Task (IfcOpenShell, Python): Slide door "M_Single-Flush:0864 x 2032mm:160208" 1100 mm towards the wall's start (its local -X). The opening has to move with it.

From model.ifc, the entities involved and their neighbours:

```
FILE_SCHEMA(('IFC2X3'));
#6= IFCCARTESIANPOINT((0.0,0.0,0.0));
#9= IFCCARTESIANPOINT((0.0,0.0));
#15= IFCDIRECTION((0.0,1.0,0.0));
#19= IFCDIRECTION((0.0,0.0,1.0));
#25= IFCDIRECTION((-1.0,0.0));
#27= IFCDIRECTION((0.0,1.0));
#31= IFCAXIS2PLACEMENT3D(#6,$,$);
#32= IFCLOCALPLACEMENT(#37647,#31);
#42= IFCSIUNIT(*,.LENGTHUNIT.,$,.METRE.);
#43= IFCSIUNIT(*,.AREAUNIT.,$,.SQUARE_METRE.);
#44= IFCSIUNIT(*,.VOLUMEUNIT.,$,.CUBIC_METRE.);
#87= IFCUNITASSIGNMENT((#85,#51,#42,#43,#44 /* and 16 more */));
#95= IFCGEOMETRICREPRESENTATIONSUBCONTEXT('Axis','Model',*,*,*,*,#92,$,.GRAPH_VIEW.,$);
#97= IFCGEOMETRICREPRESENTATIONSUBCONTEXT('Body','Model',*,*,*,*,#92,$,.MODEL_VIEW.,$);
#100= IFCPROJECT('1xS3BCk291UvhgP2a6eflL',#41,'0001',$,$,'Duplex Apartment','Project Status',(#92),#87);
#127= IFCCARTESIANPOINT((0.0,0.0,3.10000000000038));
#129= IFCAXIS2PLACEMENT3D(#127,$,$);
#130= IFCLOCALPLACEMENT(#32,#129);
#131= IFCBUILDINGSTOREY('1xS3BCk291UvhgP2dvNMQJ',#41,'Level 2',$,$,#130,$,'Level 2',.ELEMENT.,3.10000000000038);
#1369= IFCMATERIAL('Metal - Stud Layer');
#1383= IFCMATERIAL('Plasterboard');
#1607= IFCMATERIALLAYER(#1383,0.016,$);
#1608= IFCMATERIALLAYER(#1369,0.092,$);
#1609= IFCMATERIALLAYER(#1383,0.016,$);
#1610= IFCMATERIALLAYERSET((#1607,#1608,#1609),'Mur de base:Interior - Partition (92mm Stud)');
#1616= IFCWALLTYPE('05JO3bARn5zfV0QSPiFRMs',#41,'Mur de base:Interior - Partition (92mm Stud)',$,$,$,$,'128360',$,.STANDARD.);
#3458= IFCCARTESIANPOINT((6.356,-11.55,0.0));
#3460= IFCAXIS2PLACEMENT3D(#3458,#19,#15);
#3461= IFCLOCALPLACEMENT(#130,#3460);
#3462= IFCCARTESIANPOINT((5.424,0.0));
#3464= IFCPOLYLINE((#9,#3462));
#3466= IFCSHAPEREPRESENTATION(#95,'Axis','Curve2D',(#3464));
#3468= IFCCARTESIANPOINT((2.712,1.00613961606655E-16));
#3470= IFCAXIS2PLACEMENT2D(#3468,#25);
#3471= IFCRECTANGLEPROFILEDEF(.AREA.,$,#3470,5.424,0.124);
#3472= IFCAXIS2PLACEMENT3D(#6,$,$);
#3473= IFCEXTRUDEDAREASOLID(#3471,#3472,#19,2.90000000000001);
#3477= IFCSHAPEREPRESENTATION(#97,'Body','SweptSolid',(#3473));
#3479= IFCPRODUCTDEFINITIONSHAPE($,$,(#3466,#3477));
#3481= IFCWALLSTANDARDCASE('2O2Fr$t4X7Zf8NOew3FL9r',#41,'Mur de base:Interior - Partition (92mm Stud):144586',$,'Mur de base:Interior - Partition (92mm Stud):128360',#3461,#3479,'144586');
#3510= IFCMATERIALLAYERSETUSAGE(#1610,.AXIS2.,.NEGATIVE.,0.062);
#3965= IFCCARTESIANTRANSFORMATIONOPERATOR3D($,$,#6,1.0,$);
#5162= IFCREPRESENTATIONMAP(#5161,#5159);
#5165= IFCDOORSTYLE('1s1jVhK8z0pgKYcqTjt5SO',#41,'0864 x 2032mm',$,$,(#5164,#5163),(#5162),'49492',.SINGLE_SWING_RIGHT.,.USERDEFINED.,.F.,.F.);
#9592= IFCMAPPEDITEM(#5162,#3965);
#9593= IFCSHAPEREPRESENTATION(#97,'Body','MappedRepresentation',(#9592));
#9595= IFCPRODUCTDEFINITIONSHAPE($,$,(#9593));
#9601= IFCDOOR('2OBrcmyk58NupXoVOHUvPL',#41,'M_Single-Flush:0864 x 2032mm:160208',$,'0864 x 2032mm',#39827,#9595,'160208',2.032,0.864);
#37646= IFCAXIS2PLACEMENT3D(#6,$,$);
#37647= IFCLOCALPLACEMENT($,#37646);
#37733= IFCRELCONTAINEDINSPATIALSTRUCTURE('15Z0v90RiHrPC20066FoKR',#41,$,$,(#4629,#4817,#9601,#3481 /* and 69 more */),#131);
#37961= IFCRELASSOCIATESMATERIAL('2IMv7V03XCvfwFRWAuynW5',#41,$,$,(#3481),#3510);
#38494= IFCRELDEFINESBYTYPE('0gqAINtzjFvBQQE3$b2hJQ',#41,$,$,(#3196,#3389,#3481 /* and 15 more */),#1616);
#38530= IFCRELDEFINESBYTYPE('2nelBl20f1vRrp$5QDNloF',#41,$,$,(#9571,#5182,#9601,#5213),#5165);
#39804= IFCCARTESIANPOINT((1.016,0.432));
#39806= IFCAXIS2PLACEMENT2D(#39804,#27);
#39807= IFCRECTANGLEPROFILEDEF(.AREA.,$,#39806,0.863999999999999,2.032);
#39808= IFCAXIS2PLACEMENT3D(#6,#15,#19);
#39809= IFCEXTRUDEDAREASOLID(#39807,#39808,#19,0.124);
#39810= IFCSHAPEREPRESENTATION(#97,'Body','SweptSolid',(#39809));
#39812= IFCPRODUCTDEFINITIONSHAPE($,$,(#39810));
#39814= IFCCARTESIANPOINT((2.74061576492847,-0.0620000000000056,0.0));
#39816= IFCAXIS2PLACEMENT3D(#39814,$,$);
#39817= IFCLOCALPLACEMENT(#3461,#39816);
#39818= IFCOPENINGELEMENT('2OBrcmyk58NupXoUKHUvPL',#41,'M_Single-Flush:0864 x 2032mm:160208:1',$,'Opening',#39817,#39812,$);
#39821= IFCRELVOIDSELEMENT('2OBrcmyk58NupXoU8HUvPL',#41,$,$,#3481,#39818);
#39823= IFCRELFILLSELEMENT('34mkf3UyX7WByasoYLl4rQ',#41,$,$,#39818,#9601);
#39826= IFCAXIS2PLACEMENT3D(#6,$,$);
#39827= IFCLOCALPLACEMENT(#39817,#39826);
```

```python
import ifcopenshell
import ifcopenshell.api.geometry
import ifcopenshell.util.placement
import ifcopenshell.util.unit

model = ifcopenshell.open("model.ifc")
unit_scale = ifcopenshell.util.unit.calculate_unit_scale(model)

door = model.by_guid("2OBrcmyk58NupXoVOHUvPL")
opening = door.FillsVoids[0].RelatingOpeningElement
wall = opening.VoidsElements[0].RelatingBuildingElement

wall_matrix = ifcopenshell.util.placement.get_local_placement(wall.ObjectPlacement)
shift = wall_matrix[:3, 0] * -1.1 / unit_scale
before = ifcopenshell.util.placement.get_local_placement(door.ObjectPlacement)[:3, 3].copy()

# The door is placed relative to its opening, so it follows when the opening moves.
matrix = ifcopenshell.util.placement.get_local_placement(opening.ObjectPlacement)
matrix[:3, 3] += shift
ifcopenshell.api.geometry.edit_object_placement(
    model, product=opening, matrix=matrix, is_si=False, should_transform_children=True
)

after = ifcopenshell.util.placement.get_local_placement(door.ObjectPlacement)[:3, 3]
print("door moved by", (after - before).round(3) + 0.0)

model.write("model_updated.ifc")
```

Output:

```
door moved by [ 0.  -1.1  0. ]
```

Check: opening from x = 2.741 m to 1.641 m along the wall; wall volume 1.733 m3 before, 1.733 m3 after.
